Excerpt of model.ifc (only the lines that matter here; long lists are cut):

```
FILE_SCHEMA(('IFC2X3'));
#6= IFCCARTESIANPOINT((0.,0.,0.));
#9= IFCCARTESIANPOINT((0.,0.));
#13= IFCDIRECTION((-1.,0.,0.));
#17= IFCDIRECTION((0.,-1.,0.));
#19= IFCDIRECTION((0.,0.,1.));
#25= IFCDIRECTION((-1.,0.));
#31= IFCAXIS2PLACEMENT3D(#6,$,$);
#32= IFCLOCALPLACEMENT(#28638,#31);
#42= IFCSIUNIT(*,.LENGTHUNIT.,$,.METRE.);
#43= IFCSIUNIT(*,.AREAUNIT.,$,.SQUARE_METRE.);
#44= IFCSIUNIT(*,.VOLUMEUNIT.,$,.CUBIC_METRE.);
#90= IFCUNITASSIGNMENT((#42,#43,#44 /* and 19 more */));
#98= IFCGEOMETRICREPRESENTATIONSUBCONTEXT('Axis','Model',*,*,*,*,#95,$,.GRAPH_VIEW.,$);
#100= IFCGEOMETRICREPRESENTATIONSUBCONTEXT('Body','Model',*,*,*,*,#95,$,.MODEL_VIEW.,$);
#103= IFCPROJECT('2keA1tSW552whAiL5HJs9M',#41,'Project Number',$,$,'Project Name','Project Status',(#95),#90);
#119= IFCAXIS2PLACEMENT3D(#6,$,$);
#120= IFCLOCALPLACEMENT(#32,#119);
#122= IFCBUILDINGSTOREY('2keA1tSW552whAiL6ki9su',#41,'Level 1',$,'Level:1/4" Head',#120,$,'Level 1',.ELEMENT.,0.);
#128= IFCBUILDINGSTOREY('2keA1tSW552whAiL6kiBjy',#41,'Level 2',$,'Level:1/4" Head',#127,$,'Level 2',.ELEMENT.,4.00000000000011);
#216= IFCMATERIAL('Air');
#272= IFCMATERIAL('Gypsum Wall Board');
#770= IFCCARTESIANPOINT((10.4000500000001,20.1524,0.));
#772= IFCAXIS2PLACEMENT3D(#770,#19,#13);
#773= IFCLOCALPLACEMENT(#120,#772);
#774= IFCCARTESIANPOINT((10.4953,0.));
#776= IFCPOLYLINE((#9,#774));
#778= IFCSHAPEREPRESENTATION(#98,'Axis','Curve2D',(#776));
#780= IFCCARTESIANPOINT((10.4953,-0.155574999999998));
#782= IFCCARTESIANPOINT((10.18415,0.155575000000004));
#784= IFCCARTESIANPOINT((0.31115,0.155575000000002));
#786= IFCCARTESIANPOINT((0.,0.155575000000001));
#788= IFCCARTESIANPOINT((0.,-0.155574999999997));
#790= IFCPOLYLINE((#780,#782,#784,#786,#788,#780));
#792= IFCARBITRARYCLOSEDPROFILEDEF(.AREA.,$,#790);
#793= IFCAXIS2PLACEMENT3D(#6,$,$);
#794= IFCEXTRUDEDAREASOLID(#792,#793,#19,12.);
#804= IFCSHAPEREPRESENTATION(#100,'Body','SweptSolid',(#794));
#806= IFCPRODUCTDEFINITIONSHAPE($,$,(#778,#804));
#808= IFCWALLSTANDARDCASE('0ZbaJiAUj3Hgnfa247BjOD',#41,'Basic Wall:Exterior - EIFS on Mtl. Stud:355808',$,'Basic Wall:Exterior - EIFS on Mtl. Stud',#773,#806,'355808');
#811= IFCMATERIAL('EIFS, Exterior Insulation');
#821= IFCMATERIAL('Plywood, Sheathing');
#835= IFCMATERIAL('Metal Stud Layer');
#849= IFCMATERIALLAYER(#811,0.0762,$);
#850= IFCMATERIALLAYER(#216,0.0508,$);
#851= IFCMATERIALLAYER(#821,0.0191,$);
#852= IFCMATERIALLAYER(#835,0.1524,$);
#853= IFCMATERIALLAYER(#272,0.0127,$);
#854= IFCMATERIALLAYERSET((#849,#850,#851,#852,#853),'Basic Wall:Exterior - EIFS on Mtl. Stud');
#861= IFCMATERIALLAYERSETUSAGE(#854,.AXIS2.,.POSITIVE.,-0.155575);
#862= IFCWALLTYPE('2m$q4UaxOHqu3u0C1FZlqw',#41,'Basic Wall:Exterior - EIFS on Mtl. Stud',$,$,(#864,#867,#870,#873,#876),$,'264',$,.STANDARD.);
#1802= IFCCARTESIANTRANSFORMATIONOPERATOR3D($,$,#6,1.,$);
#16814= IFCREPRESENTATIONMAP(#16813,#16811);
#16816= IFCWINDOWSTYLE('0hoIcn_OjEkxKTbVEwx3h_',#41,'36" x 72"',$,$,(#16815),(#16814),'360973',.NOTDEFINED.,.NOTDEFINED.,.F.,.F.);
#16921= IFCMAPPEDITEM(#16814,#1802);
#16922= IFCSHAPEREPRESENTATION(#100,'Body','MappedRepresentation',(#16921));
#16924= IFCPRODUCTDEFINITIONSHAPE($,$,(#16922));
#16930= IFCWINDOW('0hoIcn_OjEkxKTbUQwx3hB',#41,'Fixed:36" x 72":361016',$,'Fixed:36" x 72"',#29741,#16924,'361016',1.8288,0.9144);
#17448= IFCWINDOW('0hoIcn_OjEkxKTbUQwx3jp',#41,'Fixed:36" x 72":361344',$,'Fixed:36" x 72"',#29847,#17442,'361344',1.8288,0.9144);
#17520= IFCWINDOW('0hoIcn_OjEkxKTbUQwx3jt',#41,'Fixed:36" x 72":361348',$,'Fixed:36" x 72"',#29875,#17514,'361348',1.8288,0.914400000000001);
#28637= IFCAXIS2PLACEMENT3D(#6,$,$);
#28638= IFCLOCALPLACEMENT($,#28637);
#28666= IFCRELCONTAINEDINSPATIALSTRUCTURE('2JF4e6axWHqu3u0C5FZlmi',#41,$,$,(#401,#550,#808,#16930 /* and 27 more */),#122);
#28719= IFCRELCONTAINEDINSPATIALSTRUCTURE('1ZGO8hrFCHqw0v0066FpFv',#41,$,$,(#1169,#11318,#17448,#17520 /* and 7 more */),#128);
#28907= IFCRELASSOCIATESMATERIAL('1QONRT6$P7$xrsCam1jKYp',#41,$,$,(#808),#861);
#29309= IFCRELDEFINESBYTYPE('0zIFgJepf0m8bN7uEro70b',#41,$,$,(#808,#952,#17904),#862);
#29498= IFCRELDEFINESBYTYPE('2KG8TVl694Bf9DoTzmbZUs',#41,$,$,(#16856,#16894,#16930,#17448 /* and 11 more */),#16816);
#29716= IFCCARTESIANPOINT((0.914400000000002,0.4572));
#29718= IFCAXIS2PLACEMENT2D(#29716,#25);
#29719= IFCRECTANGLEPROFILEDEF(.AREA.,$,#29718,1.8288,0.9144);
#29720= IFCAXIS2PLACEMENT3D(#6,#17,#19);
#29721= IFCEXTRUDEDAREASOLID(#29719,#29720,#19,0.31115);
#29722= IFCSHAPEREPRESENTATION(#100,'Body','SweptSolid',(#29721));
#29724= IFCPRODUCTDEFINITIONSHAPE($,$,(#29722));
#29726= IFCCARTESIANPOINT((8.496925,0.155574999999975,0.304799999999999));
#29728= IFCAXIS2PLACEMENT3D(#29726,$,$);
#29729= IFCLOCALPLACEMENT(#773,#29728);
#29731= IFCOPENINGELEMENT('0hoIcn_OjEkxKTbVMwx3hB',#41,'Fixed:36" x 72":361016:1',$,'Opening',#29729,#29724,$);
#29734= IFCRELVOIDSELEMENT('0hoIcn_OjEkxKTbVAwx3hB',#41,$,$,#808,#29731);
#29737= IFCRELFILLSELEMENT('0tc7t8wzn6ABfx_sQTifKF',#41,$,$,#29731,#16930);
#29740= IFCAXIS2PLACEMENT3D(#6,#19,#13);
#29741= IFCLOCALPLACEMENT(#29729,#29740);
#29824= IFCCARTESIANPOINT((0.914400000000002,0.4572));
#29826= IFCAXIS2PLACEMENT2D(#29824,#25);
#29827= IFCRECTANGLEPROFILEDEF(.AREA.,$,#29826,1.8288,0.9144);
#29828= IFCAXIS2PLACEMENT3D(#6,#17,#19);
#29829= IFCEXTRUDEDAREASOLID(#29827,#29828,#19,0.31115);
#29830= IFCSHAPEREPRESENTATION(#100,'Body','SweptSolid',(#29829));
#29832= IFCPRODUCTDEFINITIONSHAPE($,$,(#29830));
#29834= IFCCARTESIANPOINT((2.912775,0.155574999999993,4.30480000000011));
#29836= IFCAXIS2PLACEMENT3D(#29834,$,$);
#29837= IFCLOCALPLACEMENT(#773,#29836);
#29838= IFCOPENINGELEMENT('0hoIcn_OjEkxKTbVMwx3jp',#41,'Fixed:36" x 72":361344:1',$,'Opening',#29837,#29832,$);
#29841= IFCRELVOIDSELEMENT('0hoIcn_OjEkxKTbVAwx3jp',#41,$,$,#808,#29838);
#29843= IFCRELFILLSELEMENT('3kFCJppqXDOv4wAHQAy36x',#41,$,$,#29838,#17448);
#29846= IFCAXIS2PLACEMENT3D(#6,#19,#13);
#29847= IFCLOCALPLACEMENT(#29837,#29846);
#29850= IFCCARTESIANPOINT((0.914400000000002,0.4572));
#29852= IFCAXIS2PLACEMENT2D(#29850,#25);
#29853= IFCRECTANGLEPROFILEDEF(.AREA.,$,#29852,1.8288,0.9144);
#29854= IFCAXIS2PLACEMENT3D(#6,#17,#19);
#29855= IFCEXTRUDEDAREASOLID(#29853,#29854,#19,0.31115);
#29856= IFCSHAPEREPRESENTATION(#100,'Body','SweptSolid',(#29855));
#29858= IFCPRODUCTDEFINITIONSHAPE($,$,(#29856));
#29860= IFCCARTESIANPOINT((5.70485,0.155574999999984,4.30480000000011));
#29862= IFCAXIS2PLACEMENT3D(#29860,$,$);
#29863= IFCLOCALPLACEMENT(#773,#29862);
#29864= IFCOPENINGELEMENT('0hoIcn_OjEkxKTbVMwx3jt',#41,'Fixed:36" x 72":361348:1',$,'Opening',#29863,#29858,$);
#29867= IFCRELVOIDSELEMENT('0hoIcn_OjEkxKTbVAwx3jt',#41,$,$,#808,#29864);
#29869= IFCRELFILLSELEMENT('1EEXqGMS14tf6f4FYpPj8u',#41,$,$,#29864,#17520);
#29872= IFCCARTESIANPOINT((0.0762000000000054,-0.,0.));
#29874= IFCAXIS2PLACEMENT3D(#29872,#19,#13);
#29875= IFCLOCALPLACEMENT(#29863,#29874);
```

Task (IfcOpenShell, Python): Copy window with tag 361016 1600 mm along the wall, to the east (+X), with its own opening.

```python
import ifcopenshell
import ifcopenshell.api.feature
import ifcopenshell.api.geometry
import ifcopenshell.api.root
import ifcopenshell.geom
import ifcopenshell.util.element
import ifcopenshell.util.placement
import ifcopenshell.util.shape

model = ifcopenshell.open("model.ifc")
settings = ifcopenshell.geom.settings()


def volume(element):
    """Net volume in cubic metres, openings subtracted."""
    shape = ifcopenshell.geom.create_shape(settings, element)
    return ifcopenshell.util.shape.get_volume(shape.geometry)


def reuse_history(source, copy):
    """copy_class also copies each property set's owner history, people and application; keep the originals."""
    for rel in copy.IsDefinedBy:
        if rel.is_a("IfcRelDefinesByProperties") and (history := rel.RelatingPropertyDefinition.OwnerHistory):
            rel.RelatingPropertyDefinition.OwnerHistory = source.OwnerHistory
            ifcopenshell.util.element.remove_deep2(model, history)


window = model.by_guid("0hoIcn_OjEkxKTbUQwx3hB")
opening = window.FillsVoids[0].RelatingOpeningElement
wall = opening.VoidsElements[0].RelatingBuildingElement
before = volume(wall)
shift = ifcopenshell.util.placement.get_local_placement(wall.ObjectPlacement)[:3, 0] * -1.6

# copy_class copies the void relationship, type, container and properties, but no geometry.
new_opening = ifcopenshell.api.root.copy_class(model, product=opening)
new_opening.Representation = ifcopenshell.util.element.copy_deep(
    model, opening.Representation, exclude=["IfcGeometricRepresentationContext", "IfcRepresentationMap"]
)
new_opening.Name = 'Fixed:36" x 72"'
new_window = ifcopenshell.api.root.copy_class(model, product=window)
new_window.Representation = ifcopenshell.util.element.copy_deep(
    model, window.Representation, exclude=["IfcGeometricRepresentationContext", "IfcRepresentationMap"]
)
new_window.Name = 'Fixed:36" x 72"'
new_window.Tag = None
reuse_history(window, new_window)
fills = ifcopenshell.api.feature.add_filling(model, opening=new_opening, element=new_window)
fills.OwnerHistory = new_window.OwnerHistory  # required in IFC2X3

for old, new in ((opening, new_opening), (window, new_window)):
    matrix = ifcopenshell.util.placement.get_local_placement(old.ObjectPlacement)
    matrix[:3, 3] += shift
    ifcopenshell.api.geometry.edit_object_placement(model, product=new, matrix=matrix, is_si=False)

after = volume(wall)

print(f"wall volume {before:.3f} -> {after:.3f} m3")

model.write("model_updated.ifc")
```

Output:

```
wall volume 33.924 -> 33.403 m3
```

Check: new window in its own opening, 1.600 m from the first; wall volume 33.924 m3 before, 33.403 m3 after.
